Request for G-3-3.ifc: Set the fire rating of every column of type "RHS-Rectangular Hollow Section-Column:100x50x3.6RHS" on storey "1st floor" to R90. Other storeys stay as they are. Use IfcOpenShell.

First a look at what the model holds.

```python
import ifcopenshell
import ifcopenshell.util.element

model = ifcopenshell.open("G-3-3.ifc")
print(model.schema)
storey = next(s for s in model.by_type("IfcBuildingStorey") if s.Name == "1st floor")
columns = [e for e in ifcopenshell.util.element.get_decomposition(storey) if e.is_a("IfcColumn")]
seen = {}
for e in columns:
    element_type = ifcopenshell.util.element.get_type(e)
    key = (element_type.Name if element_type != e and element_type else None, ifcopenshell.util.element.get_pset(e, "Pset_ColumnCommon", "FireRating"))
    seen[key] = seen.get(key, 0) + 1
for (name, value), count in sorted(seen.items(), key=str):
    print(count, "x", name, "|", value)
```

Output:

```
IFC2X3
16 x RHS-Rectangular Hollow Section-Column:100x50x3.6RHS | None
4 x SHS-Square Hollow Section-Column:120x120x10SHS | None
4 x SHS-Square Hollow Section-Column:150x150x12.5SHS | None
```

```python
import ifcopenshell
import ifcopenshell.api.pset
import ifcopenshell.util.element

model = ifcopenshell.open("G-3-3.ifc")

storey = next(s for s in model.by_type("IfcBuildingStorey") if s.Name == "1st floor")
columns = [e for e in ifcopenshell.util.element.get_decomposition(storey) if e.is_a("IfcColumn")]

count = 0
for e in columns:
    element_type = ifcopenshell.util.element.get_type(e)
    if element_type in (None, e) or element_type.Name != "RHS-Rectangular Hollow Section-Column:100x50x3.6RHS":
        continue
    # add_pset returns the element's existing set when there is one.
    pset = ifcopenshell.api.pset.add_pset(model, product=e, name="Pset_ColumnCommon")
    ifcopenshell.api.pset.edit_pset(model, pset=pset, properties={"FireRating": "R90"})
    count += 1

print(count, "columns updated")

model.write("G-3-3_v2.ifc")
```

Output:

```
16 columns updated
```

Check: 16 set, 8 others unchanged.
